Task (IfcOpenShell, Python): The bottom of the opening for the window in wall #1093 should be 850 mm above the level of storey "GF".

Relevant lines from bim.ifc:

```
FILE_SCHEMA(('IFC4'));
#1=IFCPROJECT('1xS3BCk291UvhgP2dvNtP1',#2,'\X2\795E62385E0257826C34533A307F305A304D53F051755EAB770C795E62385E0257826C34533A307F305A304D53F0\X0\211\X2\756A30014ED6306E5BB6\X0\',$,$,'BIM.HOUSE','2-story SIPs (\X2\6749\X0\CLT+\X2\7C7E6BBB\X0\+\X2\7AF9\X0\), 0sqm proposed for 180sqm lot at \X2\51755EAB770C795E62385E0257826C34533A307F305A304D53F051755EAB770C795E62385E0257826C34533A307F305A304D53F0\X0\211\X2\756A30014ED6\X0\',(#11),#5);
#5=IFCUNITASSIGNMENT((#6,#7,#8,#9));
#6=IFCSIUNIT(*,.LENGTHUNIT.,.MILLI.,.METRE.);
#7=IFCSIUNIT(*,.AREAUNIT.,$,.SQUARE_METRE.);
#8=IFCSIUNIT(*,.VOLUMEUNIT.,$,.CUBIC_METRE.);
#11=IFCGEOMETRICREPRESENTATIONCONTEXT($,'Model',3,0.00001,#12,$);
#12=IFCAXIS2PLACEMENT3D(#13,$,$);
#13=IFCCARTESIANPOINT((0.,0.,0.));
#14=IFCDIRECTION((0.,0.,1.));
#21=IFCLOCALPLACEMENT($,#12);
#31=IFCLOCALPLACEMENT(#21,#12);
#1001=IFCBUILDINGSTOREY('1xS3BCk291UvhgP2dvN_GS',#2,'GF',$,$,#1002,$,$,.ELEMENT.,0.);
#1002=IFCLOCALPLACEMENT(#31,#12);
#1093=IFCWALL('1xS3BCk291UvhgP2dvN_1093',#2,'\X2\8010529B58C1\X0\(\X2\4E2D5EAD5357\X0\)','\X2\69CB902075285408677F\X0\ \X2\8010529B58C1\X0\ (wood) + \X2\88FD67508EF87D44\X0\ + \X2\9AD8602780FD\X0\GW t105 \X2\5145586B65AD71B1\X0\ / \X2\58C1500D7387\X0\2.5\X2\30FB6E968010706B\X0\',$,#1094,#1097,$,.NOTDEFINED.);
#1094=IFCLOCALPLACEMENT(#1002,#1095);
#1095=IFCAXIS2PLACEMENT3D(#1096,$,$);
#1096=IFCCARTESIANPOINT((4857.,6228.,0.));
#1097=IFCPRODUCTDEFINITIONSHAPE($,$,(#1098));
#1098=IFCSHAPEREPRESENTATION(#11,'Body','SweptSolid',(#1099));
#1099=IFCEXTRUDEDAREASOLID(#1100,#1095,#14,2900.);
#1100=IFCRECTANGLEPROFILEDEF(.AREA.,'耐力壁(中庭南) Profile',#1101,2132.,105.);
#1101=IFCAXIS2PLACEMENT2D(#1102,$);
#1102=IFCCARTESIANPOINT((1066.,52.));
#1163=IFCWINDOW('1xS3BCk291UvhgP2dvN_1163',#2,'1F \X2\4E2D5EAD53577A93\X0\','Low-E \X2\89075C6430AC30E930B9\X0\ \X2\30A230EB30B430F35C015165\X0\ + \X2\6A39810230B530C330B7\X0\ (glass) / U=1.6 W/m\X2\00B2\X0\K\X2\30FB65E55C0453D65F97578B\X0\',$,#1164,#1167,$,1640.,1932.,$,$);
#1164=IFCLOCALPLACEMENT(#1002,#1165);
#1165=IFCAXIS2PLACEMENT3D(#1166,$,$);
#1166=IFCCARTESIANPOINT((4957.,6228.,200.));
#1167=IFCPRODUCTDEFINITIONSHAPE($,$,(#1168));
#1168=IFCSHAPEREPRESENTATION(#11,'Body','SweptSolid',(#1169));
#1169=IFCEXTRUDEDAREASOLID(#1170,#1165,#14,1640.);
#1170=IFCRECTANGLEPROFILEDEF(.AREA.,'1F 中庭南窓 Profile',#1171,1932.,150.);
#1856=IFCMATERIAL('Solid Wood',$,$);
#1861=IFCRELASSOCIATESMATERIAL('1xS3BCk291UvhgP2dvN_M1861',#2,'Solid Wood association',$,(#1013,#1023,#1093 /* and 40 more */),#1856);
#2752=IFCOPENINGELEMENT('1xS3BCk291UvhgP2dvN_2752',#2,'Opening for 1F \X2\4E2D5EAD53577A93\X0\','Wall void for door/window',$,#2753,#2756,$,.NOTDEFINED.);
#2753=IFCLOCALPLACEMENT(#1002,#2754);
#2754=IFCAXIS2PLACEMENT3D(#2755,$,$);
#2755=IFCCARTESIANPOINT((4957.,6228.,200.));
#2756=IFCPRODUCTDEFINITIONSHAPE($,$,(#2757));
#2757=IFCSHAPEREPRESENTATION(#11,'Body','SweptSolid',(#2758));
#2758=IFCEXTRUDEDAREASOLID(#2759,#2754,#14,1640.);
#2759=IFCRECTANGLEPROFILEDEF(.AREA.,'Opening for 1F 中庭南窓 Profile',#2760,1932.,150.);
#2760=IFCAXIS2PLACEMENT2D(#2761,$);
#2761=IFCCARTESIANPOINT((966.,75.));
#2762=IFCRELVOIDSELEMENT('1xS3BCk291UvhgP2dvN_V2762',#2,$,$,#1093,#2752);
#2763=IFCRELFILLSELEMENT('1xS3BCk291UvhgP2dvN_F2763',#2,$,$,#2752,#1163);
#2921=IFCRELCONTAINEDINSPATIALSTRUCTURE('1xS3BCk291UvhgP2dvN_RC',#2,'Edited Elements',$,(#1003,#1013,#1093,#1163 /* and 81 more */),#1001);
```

```python
import numpy as np
import ifcopenshell
import ifcopenshell.api.geometry
import ifcopenshell.geom
import ifcopenshell.util.element
import ifcopenshell.util.placement
import ifcopenshell.util.shape
import ifcopenshell.util.unit

model = ifcopenshell.open("bim.ifc")
unit_scale = ifcopenshell.util.unit.calculate_unit_scale(model)

window = model.by_id(1163)
opening = window.FillsVoids[0].RelatingOpeningElement
storey = ifcopenshell.util.element.get_container(window, ifc_class="IfcBuildingStorey")
level = ifcopenshell.util.placement.get_local_placement(storey.ObjectPlacement)[2, 3]

# The opening's origin need not be at the sill, so measure its lowest point.
shape = ifcopenshell.geom.create_shape(ifcopenshell.geom.settings(), opening)
bottom = ifcopenshell.util.shape.get_shape_bottom_elevation(shape, shape.geometry) / unit_scale
dz = level + 0.85 / unit_scale - bottom

shift = np.array([0.0, 0.0, dz])
# The window is not placed relative to its opening, so move both.
for product in (opening, window):
    matrix = ifcopenshell.util.placement.get_local_placement(product.ObjectPlacement)
    matrix[:3, 3] += shift
    ifcopenshell.api.geometry.edit_object_placement(model, product=product, matrix=matrix, is_si=False)

print(f"moved by {dz * unit_scale:+.3f} m")

model.write("bim_v2.ifc")
```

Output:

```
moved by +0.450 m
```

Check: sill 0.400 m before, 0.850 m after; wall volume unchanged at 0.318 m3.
